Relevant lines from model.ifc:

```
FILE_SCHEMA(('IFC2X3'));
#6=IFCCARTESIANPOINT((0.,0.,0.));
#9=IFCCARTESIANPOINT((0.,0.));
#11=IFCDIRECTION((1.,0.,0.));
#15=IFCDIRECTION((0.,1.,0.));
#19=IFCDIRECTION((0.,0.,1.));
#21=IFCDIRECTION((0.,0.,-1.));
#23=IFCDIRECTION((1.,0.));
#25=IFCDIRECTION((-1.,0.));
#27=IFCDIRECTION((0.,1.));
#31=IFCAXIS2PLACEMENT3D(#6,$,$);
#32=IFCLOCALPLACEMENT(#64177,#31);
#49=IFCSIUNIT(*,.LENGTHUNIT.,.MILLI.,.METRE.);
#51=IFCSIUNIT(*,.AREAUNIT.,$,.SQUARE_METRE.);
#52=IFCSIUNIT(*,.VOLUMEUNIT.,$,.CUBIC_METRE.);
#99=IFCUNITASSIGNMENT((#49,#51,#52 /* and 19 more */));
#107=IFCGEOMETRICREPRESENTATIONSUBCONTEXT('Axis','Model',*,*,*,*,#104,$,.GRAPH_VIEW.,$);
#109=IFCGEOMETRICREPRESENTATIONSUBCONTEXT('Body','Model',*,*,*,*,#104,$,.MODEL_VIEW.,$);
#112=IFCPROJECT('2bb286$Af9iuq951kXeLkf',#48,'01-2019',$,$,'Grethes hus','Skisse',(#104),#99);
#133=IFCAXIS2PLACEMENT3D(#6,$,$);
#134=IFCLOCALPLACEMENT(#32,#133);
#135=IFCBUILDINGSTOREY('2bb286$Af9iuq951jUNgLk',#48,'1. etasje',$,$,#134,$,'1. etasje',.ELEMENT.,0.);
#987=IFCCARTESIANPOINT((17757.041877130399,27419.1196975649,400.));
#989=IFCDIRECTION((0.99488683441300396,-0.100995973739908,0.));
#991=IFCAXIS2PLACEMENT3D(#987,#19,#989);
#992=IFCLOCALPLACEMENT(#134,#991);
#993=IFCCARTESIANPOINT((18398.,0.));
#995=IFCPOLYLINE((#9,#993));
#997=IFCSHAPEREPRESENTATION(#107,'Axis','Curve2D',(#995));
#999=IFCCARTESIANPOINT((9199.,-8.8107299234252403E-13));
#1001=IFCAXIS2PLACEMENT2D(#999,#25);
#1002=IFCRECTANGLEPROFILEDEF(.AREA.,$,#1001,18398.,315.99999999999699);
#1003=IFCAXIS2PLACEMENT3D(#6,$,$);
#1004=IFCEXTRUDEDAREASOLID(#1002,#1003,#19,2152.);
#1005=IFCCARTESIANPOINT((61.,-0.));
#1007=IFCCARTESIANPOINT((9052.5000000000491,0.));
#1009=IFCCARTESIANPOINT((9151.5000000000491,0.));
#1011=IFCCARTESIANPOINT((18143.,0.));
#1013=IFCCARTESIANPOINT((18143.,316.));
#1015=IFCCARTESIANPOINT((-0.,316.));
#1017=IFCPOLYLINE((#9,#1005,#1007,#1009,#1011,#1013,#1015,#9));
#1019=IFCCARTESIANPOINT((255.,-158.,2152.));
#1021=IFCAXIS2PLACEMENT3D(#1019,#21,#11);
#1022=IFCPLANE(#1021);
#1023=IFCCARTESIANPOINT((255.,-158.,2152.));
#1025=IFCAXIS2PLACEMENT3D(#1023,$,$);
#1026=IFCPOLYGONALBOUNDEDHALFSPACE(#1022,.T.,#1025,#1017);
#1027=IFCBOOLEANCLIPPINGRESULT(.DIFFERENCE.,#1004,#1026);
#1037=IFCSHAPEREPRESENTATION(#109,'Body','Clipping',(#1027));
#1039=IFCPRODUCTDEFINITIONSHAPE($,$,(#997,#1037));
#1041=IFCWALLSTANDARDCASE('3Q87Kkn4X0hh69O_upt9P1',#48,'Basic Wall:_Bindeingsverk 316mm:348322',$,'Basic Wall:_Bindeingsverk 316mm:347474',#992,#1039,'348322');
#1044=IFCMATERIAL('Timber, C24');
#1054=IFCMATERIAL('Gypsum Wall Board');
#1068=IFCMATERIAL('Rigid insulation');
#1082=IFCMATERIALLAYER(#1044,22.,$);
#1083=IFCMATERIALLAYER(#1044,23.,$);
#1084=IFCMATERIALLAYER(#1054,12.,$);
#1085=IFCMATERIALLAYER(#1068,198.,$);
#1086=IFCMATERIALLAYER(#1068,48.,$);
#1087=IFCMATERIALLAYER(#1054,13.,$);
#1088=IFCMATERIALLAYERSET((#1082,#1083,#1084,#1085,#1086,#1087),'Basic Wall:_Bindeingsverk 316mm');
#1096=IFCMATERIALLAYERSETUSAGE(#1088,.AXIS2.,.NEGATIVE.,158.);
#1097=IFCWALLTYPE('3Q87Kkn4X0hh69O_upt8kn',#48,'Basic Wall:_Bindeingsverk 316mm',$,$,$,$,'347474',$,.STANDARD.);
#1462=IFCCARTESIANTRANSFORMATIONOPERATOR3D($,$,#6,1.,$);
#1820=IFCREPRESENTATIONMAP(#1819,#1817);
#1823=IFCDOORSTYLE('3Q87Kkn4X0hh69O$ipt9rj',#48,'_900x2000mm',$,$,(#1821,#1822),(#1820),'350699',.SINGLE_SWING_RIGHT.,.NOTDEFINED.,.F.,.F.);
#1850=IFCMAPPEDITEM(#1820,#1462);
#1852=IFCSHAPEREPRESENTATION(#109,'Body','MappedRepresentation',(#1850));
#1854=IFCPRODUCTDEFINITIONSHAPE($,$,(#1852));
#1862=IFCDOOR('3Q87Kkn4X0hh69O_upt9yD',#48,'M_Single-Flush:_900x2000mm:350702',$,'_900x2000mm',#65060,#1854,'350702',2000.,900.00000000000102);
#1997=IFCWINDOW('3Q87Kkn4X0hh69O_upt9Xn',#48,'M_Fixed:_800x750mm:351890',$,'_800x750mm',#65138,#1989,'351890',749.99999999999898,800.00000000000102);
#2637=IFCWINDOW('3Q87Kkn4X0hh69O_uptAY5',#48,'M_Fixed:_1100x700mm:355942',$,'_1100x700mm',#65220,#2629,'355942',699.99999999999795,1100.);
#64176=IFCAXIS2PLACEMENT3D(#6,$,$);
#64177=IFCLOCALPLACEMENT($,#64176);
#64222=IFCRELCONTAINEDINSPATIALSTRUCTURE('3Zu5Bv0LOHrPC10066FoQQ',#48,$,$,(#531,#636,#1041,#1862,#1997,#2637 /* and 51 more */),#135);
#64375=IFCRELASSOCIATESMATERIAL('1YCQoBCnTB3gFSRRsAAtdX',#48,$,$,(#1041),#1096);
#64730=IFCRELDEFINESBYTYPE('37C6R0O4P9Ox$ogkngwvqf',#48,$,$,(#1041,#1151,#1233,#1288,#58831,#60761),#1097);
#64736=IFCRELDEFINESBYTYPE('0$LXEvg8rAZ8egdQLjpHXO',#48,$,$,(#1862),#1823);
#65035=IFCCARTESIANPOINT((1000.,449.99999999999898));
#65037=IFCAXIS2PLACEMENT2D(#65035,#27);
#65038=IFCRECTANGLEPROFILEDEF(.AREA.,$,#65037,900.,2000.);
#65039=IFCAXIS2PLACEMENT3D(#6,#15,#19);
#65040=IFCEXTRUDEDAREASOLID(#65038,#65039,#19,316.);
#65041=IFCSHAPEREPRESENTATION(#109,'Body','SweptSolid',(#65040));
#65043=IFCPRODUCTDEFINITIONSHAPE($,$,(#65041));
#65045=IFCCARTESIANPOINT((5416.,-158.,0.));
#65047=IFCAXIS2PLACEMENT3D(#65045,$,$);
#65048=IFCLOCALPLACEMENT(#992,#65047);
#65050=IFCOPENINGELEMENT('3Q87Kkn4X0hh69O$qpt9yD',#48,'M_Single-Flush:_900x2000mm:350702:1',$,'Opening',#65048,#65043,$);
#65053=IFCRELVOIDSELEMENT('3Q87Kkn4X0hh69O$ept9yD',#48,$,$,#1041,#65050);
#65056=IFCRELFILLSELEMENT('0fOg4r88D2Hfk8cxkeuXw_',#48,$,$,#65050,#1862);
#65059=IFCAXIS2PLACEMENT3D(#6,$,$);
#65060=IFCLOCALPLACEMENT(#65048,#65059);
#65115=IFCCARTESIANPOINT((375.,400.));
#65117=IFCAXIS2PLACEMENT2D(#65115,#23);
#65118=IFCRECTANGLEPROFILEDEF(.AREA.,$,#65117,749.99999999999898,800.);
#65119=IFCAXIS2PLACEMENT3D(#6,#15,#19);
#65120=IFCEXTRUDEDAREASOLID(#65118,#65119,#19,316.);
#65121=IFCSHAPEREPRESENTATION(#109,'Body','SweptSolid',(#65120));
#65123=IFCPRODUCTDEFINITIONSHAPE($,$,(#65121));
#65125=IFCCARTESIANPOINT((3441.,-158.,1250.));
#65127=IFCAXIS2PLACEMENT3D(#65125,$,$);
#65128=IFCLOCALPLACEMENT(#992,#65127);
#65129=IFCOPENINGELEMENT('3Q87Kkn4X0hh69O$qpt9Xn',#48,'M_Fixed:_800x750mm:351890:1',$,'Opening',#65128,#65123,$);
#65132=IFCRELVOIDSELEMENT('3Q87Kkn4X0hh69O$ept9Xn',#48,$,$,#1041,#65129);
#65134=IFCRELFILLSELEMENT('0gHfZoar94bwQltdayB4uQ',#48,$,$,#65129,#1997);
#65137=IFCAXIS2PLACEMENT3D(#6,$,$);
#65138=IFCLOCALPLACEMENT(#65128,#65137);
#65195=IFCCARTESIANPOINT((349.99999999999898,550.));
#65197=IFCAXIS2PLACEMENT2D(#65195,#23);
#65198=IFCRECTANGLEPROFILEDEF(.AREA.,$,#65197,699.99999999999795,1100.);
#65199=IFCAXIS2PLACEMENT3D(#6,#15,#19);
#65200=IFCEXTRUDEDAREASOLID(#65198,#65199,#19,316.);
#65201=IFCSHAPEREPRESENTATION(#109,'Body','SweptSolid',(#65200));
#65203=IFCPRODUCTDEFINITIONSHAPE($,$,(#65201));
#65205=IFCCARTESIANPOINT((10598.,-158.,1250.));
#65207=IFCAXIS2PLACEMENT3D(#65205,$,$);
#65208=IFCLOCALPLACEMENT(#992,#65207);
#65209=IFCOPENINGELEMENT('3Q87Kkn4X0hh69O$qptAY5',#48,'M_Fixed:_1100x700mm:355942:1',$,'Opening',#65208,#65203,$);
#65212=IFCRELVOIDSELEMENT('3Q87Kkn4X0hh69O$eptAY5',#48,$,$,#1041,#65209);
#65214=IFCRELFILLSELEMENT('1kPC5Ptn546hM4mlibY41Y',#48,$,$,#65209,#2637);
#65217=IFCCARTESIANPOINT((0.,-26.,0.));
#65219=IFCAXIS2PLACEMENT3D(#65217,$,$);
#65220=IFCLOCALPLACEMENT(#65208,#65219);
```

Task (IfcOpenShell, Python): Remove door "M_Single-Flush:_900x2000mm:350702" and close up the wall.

```python
import ifcopenshell
import ifcopenshell.api.feature
import ifcopenshell.api.root
import ifcopenshell.geom
import ifcopenshell.util.shape

model = ifcopenshell.open("model.ifc")
settings = ifcopenshell.geom.settings()


def volume(element):
    """Net volume in cubic metres, openings subtracted."""
    shape = ifcopenshell.geom.create_shape(settings, element)
    return ifcopenshell.util.shape.get_volume(shape.geometry)


door = model.by_guid("3Q87Kkn4X0hh69O_upt9yD")
opening = door.FillsVoids[0].RelatingOpeningElement
wall = opening.VoidsElements[0].RelatingBuildingElement
before = volume(wall)

ifcopenshell.api.root.remove_product(model, product=door)
ifcopenshell.api.feature.remove_feature(model, feature=opening)

after = volume(wall)

print(f"wall volume {before:.3f} -> {after:.3f} m3")

model.write("model-out.ifc")
```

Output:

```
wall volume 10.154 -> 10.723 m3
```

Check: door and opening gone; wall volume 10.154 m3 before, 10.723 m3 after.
